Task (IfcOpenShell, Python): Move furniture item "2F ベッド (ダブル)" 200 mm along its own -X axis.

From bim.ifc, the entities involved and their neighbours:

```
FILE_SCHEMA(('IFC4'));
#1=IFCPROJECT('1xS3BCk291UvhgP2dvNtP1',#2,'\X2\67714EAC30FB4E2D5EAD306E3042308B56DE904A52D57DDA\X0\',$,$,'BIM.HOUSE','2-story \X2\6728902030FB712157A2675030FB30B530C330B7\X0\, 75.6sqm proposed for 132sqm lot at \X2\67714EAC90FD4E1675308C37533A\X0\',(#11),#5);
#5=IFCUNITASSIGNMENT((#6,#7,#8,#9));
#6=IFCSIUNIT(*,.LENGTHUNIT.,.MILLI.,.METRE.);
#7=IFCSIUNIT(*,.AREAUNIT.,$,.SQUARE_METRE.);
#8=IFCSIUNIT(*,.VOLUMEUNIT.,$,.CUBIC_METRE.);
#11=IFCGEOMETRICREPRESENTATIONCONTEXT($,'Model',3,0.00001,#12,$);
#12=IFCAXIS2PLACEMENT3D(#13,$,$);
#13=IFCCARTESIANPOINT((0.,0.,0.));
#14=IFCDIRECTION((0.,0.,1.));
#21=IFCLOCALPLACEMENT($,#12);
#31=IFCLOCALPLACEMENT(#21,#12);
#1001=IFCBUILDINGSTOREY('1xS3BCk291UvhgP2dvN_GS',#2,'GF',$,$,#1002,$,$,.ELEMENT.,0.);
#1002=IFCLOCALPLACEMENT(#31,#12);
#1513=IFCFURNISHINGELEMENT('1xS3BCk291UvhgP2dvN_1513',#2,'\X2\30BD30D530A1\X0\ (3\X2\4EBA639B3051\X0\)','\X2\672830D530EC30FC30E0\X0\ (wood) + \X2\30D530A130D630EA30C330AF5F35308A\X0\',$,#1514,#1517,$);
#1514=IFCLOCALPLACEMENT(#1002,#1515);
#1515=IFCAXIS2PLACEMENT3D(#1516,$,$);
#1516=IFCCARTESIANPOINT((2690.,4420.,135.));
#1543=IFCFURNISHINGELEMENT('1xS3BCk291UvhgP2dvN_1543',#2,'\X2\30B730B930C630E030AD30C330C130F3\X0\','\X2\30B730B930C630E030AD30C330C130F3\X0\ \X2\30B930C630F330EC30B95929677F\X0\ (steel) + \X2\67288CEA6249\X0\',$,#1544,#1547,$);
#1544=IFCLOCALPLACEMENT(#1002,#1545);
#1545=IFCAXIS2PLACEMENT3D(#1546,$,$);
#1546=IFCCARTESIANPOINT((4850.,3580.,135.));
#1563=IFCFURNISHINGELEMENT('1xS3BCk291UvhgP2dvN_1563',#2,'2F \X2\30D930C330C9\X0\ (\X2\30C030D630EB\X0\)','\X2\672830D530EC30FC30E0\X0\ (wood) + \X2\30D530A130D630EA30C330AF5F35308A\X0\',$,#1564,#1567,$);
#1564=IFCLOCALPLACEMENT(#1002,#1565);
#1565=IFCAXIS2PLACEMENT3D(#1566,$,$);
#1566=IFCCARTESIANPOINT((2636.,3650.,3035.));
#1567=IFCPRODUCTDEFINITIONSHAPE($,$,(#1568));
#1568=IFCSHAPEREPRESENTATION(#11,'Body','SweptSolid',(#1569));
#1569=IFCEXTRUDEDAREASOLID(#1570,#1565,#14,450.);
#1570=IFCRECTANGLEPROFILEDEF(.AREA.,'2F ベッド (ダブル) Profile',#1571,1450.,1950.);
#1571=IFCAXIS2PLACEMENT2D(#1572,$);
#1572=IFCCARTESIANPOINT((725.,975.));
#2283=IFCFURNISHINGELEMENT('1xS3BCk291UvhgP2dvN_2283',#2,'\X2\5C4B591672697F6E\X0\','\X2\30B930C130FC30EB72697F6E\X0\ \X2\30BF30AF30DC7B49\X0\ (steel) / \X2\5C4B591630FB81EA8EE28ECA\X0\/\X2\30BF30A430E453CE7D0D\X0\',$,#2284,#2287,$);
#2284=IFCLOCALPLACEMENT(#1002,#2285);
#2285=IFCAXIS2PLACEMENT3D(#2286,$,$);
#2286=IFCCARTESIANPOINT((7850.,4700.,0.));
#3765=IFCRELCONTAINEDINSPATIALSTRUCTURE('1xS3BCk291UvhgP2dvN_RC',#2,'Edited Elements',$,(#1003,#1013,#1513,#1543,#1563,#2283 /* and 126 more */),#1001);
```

```python
import ifcopenshell
import ifcopenshell.api.geometry
import ifcopenshell.util.placement

model = ifcopenshell.open("bim.ifc")

item = model.by_id(1563)
matrix = ifcopenshell.util.placement.get_local_placement(item.ObjectPlacement)
matrix[:3, 3] -= matrix[:3, 0] * 200.0
ifcopenshell.api.geometry.edit_object_placement(model, product=item, matrix=matrix, is_si=False)

print(ifcopenshell.util.placement.get_local_placement(item.ObjectPlacement).round(3) + 0.0)

model.write("bim_updated.ifc")
```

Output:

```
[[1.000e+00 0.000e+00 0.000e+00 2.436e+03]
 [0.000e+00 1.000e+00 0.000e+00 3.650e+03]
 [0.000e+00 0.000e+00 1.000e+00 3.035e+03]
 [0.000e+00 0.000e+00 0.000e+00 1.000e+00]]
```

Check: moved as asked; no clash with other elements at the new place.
